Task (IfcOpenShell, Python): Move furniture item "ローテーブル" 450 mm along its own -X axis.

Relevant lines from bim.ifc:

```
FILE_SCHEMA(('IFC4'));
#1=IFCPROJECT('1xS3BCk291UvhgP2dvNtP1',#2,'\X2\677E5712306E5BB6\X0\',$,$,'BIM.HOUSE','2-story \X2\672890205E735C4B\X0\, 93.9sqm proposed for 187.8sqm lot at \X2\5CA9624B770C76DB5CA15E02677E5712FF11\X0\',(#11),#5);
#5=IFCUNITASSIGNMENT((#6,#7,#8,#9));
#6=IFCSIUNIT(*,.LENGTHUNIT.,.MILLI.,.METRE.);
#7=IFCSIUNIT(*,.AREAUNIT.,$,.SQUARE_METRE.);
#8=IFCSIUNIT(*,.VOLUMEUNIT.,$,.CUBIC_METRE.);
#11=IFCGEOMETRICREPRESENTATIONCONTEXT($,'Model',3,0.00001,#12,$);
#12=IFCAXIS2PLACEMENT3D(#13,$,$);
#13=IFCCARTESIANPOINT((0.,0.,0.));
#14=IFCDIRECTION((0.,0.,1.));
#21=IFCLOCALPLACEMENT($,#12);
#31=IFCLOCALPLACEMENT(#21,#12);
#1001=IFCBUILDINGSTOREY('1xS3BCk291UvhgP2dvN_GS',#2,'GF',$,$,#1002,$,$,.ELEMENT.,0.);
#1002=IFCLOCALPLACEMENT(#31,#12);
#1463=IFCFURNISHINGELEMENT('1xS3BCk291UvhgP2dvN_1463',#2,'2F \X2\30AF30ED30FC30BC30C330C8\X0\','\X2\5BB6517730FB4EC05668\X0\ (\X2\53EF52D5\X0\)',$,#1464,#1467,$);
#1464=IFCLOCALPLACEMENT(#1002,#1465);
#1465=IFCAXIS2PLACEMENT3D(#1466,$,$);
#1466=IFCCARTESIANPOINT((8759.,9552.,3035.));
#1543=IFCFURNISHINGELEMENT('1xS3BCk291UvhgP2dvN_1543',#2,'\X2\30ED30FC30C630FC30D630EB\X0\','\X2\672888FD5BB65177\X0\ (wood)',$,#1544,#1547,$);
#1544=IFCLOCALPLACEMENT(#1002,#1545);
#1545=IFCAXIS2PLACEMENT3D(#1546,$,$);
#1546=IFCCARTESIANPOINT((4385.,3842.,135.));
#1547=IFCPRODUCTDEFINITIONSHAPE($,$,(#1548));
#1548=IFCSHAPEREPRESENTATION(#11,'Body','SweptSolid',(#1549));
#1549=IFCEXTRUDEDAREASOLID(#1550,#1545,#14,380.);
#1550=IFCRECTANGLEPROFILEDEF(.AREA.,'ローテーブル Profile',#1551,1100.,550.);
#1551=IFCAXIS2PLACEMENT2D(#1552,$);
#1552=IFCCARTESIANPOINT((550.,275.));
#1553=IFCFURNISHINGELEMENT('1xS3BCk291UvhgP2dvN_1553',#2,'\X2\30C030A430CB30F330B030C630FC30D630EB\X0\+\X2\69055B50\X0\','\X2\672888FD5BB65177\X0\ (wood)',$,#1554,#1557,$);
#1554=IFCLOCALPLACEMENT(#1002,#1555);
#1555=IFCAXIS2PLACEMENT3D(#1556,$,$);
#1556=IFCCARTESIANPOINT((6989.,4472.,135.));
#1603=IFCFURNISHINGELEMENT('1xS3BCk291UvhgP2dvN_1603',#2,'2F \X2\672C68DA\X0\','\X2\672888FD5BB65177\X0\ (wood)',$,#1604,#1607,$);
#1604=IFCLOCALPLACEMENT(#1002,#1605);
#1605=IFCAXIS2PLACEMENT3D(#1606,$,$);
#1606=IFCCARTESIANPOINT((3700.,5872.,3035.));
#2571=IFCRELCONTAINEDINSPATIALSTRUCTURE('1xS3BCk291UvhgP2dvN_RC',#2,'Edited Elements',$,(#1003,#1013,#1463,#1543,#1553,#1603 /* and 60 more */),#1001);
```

```python
import ifcopenshell
import ifcopenshell.api.geometry
import ifcopenshell.util.placement
import ifcopenshell.util.unit

model = ifcopenshell.open("bim.ifc")
unit_scale = ifcopenshell.util.unit.calculate_unit_scale(model)

item = model.by_guid("1xS3BCk291UvhgP2dvN_1543")
matrix = ifcopenshell.util.placement.get_local_placement(item.ObjectPlacement)
matrix[:3, 3] -= matrix[:3, 0] * 0.45 / unit_scale
ifcopenshell.api.geometry.edit_object_placement(model, product=item, matrix=matrix, is_si=False)

print(ifcopenshell.util.placement.get_local_placement(item.ObjectPlacement).round(3) + 0.0)

model.write("bim_updated.ifc")
```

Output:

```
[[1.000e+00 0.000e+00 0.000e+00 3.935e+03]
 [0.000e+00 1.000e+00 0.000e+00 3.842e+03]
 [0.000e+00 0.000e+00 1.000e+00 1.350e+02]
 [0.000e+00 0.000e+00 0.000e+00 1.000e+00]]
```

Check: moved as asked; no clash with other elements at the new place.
